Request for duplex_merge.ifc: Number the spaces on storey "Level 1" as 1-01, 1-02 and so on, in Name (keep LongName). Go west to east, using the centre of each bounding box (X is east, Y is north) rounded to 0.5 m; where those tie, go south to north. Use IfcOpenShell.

First a look at what the model holds.

```python
import ifcopenshell
import ifcopenshell.util.element
import ifcopenshell.util.placement

model = ifcopenshell.open("duplex_merge.ifc")
print(model.schema)
storey = next(s for s in model.by_type("IfcBuildingStorey") if s.Name == "Level 1")
spaces = [e for e in ifcopenshell.util.element.get_decomposition(storey) if e.is_a("IfcSpace")]
for e in sorted(spaces, key=lambda e: e.id()):
    origin = ifcopenshell.util.placement.get_local_placement(e.ObjectPlacement)[:3, 3]
    print(e.id(), e.Name, e.LongName, origin.round(2) + 0.0, sep=" | ")
```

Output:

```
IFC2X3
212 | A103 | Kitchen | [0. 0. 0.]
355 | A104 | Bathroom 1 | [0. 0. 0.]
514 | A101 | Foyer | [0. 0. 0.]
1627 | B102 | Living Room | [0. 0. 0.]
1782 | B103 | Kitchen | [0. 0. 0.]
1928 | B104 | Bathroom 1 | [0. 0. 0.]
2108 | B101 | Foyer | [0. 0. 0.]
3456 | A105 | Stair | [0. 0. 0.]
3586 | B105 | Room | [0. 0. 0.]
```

```python
import ifcopenshell
import ifcopenshell.geom
import ifcopenshell.util.element
import ifcopenshell.util.shape

model = ifcopenshell.open("duplex_merge.ifc")
settings = ifcopenshell.geom.settings()
settings.set("use-world-coords", True)


def centre(element):
    shape = ifcopenshell.geom.create_shape(settings, element)
    return ifcopenshell.util.shape.get_bbox_centroid(shape.geometry)


storey = next(s for s in model.by_type("IfcBuildingStorey") if s.Name == "Level 1")
spaces = [e for e in ifcopenshell.util.element.get_decomposition(storey) if e.is_a("IfcSpace")]

# Insertion points can sit at a corner or the storey origin, so sort by the geometry (in metres).
centres = {e: centre(e) for e in spaces}
spaces.sort(key=lambda e: (round(centres[e][0] / 0.5), centres[e][1]))

for i, e in enumerate(spaces, start=1):
    number = f"1-{i:02d}"
    e.Name = number
    print(e.id(), number)

model.write("duplex_merge_updated.ifc")
```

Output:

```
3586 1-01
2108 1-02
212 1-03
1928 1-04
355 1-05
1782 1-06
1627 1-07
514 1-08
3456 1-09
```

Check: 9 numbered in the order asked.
